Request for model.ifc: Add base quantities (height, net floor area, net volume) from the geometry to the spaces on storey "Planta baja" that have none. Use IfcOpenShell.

First a look at what the model holds.

```python
import ifcopenshell
import ifcopenshell.util.element
import ifcopenshell.util.unit

model = ifcopenshell.open("model.ifc")
print(model.schema)
for unit_type in ("LENGTHUNIT", "AREAUNIT", "VOLUMEUNIT"):
    print(unit_type, ifcopenshell.util.unit.calculate_unit_scale(model, unit_type))
storey = next(s for s in model.by_type("IfcBuildingStorey") if s.Name == "Planta baja")
spaces = [e for e in ifcopenshell.util.element.get_decomposition(storey) if e.is_a("IfcSpace")]
for e in sorted(spaces, key=lambda e: e.id()):
    print(e.id(), e.is_a(), e.Name, list(ifcopenshell.util.element.get_psets(e, qtos_only=True)), sep=" | ")
```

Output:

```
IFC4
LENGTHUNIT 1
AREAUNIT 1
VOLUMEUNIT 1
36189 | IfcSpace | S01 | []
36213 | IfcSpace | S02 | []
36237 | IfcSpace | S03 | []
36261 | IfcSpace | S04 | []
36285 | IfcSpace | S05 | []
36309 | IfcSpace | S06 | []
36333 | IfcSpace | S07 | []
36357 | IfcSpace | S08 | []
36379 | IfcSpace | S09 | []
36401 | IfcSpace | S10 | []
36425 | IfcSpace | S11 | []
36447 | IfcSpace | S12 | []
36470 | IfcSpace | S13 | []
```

```python
import ifcopenshell
import ifcopenshell.api.pset
import ifcopenshell.geom
import ifcopenshell.util.element
import ifcopenshell.util.shape
import ifcopenshell.util.unit

model = ifcopenshell.open("model.ifc")
unit_scale = ifcopenshell.util.unit.calculate_unit_scale(model)
area_scale = ifcopenshell.util.unit.calculate_unit_scale(model, "AREAUNIT")
volume_scale = ifcopenshell.util.unit.calculate_unit_scale(model, "VOLUMEUNIT")
settings = ifcopenshell.geom.settings()

storey = next(s for s in model.by_type("IfcBuildingStorey") if s.Name == "Planta baja")
spaces = [e for e in ifcopenshell.util.element.get_decomposition(storey) if e.is_a("IfcSpace")]

for e in sorted(spaces, key=lambda e: e.id()):
    if ifcopenshell.util.element.get_psets(e, qtos_only=True, should_inherit=False):
        continue
    # Geometry comes back in metres, in the element's own axes.
    shape = ifcopenshell.geom.create_shape(settings, e)
    values = {
        "Height": ifcopenshell.util.shape.get_z(shape.geometry) / unit_scale,
        "NetFloorArea": ifcopenshell.util.shape.get_footprint_area(shape.geometry) / area_scale,
        "NetVolume": ifcopenshell.util.shape.get_volume(shape.geometry) / volume_scale,
    }
    qto = ifcopenshell.api.pset.add_qto(model, product=e, name="Qto_SpaceBaseQuantities")
    ifcopenshell.api.pset.edit_qto(model, qto=qto, properties=values)
    print(e.id(), {k: round(v, 3) for k, v in values.items()})

model.write("model_edited.ifc")
```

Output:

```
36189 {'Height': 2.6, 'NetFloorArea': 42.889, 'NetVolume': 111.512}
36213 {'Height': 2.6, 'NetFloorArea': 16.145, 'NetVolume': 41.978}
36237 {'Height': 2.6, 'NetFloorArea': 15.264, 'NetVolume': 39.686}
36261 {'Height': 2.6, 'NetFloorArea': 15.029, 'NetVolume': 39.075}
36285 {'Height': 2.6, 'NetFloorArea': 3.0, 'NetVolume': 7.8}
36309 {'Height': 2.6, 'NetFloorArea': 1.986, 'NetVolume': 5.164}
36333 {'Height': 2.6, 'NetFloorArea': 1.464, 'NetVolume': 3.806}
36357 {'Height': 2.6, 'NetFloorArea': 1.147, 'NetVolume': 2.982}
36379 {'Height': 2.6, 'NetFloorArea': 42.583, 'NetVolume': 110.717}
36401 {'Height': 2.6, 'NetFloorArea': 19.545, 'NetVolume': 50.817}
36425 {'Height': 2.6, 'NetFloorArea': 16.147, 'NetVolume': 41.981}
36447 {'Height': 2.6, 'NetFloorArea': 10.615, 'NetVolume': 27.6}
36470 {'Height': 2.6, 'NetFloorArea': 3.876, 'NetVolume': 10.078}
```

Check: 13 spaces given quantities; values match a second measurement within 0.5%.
